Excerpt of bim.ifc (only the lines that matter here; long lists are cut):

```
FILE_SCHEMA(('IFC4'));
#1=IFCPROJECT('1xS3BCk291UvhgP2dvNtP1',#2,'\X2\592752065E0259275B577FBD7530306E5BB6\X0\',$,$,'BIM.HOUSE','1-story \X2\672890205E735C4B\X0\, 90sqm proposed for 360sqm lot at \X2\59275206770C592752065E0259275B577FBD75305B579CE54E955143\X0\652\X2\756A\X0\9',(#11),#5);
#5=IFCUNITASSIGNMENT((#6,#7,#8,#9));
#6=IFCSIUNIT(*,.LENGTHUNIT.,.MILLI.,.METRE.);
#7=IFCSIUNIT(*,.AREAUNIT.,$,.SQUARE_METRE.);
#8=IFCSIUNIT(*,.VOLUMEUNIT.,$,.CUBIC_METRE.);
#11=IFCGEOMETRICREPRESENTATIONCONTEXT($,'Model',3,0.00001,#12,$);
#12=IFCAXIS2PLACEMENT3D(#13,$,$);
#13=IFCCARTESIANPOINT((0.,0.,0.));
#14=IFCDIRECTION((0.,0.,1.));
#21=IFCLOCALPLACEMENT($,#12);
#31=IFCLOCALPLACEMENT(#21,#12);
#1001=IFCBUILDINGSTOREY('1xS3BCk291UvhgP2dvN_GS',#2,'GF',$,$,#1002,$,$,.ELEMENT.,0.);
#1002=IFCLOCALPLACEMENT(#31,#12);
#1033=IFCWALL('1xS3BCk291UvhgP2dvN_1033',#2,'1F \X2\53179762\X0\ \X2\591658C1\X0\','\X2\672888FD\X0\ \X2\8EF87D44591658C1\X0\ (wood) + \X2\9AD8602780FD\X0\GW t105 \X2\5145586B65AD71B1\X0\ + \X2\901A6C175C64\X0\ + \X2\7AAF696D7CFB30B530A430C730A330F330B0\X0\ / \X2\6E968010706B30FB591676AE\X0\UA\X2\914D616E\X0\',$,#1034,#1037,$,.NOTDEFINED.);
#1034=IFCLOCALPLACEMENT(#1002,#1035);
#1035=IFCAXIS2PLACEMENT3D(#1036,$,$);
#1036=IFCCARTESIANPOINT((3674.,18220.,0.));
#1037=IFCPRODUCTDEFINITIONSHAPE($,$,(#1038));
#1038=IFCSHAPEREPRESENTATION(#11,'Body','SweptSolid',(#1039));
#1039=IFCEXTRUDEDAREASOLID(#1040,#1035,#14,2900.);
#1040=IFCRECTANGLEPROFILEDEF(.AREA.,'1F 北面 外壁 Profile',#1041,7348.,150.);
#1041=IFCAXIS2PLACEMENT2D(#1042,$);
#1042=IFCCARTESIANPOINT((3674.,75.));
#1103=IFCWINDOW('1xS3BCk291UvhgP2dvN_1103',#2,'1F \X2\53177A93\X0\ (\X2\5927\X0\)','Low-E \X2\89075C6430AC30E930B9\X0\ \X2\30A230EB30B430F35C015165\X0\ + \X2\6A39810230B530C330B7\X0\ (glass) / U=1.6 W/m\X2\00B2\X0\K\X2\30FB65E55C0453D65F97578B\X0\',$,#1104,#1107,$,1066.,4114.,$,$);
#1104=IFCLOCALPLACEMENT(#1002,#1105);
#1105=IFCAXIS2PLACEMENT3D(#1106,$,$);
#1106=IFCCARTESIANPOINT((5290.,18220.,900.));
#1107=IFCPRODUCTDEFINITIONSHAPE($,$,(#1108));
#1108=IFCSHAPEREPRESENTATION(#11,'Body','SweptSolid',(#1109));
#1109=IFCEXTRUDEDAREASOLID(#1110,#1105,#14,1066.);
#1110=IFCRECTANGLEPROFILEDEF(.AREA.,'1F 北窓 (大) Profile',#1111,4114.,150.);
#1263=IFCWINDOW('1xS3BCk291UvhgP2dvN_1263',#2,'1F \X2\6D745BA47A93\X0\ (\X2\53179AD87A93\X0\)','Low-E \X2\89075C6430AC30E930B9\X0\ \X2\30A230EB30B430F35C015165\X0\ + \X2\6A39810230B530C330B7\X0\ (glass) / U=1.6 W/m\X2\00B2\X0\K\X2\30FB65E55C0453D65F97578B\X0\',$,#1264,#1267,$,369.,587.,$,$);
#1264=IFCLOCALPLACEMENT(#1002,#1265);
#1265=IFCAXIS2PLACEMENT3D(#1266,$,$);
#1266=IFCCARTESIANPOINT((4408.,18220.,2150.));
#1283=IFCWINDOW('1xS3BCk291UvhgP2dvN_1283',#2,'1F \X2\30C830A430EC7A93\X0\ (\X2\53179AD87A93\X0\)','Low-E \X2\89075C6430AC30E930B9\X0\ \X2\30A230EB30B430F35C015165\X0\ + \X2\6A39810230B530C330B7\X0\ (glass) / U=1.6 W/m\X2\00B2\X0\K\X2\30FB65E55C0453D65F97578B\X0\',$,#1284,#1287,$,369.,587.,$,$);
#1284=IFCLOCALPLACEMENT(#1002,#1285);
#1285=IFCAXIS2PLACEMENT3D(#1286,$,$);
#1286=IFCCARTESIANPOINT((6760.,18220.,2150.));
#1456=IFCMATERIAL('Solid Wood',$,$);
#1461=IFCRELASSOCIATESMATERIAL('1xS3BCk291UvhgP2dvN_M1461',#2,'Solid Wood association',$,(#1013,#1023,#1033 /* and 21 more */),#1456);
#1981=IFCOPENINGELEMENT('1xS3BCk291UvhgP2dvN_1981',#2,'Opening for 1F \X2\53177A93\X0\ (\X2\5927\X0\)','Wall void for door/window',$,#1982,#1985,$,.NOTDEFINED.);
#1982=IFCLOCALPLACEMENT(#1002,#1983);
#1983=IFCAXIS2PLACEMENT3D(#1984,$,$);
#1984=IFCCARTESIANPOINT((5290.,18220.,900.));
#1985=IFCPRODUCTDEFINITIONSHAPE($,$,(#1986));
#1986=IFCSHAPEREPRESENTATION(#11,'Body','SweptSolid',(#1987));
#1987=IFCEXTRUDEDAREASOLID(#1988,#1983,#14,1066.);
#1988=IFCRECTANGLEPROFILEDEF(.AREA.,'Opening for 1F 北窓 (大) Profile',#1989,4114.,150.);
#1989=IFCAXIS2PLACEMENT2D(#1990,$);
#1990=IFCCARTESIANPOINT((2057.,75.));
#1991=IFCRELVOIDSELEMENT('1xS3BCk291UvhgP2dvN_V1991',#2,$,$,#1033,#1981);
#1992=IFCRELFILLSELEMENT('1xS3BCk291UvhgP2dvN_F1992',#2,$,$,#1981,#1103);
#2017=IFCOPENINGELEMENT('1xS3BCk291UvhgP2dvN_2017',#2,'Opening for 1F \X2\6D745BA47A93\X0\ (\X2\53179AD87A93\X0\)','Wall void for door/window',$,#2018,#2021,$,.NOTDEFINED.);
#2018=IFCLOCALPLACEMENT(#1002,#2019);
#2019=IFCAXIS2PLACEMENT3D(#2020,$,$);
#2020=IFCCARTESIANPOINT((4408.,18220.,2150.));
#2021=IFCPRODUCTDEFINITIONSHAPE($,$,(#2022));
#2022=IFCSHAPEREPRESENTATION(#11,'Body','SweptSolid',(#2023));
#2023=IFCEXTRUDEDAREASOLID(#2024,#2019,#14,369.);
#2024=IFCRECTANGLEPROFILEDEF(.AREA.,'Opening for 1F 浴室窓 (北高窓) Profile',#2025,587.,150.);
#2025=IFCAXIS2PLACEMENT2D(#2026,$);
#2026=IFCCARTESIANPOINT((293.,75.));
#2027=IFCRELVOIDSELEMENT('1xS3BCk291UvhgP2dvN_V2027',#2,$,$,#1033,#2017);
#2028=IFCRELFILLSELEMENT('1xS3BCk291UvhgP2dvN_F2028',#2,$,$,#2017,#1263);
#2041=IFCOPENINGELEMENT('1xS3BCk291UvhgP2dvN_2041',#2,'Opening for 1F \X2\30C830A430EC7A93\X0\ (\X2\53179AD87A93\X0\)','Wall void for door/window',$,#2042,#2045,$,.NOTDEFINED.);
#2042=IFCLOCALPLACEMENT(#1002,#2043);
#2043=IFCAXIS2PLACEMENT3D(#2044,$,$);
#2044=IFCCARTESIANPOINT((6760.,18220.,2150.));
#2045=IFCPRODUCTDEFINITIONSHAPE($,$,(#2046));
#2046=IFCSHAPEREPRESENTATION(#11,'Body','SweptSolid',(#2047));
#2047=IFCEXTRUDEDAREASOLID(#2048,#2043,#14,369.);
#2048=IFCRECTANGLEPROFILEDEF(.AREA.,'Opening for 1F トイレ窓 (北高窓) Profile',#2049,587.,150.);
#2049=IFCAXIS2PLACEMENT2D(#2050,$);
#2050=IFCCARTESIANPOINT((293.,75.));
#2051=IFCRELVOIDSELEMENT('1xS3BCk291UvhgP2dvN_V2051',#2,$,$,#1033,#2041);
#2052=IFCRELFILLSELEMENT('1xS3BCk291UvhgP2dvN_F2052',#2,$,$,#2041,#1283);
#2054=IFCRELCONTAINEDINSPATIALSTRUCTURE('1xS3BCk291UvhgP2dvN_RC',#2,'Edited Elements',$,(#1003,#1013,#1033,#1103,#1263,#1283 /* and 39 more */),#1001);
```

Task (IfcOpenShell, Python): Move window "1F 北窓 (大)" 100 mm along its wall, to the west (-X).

```python
import ifcopenshell
import ifcopenshell.api.geometry
import ifcopenshell.util.placement
import ifcopenshell.util.unit

model = ifcopenshell.open("bim.ifc")
unit_scale = ifcopenshell.util.unit.calculate_unit_scale(model)

window = model.by_guid("1xS3BCk291UvhgP2dvN_1103")
opening = window.FillsVoids[0].RelatingOpeningElement
wall = opening.VoidsElements[0].RelatingBuildingElement

wall_matrix = ifcopenshell.util.placement.get_local_placement(wall.ObjectPlacement)
shift = wall_matrix[:3, 0] * -0.1 / unit_scale
before = ifcopenshell.util.placement.get_local_placement(window.ObjectPlacement)[:3, 3].copy()

# The window is not placed relative to its opening, so move both.
for product in (opening, window):
    matrix = ifcopenshell.util.placement.get_local_placement(product.ObjectPlacement)
    matrix[:3, 3] += shift
    ifcopenshell.api.geometry.edit_object_placement(model, product=product, matrix=matrix, is_si=False)

after = ifcopenshell.util.placement.get_local_placement(window.ObjectPlacement)[:3, 3]
print("window moved by", (after - before).round(3) + 0.0)

model.write("bim-out.ifc")
```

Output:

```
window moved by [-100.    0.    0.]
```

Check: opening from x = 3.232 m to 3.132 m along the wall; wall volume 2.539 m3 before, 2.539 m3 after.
